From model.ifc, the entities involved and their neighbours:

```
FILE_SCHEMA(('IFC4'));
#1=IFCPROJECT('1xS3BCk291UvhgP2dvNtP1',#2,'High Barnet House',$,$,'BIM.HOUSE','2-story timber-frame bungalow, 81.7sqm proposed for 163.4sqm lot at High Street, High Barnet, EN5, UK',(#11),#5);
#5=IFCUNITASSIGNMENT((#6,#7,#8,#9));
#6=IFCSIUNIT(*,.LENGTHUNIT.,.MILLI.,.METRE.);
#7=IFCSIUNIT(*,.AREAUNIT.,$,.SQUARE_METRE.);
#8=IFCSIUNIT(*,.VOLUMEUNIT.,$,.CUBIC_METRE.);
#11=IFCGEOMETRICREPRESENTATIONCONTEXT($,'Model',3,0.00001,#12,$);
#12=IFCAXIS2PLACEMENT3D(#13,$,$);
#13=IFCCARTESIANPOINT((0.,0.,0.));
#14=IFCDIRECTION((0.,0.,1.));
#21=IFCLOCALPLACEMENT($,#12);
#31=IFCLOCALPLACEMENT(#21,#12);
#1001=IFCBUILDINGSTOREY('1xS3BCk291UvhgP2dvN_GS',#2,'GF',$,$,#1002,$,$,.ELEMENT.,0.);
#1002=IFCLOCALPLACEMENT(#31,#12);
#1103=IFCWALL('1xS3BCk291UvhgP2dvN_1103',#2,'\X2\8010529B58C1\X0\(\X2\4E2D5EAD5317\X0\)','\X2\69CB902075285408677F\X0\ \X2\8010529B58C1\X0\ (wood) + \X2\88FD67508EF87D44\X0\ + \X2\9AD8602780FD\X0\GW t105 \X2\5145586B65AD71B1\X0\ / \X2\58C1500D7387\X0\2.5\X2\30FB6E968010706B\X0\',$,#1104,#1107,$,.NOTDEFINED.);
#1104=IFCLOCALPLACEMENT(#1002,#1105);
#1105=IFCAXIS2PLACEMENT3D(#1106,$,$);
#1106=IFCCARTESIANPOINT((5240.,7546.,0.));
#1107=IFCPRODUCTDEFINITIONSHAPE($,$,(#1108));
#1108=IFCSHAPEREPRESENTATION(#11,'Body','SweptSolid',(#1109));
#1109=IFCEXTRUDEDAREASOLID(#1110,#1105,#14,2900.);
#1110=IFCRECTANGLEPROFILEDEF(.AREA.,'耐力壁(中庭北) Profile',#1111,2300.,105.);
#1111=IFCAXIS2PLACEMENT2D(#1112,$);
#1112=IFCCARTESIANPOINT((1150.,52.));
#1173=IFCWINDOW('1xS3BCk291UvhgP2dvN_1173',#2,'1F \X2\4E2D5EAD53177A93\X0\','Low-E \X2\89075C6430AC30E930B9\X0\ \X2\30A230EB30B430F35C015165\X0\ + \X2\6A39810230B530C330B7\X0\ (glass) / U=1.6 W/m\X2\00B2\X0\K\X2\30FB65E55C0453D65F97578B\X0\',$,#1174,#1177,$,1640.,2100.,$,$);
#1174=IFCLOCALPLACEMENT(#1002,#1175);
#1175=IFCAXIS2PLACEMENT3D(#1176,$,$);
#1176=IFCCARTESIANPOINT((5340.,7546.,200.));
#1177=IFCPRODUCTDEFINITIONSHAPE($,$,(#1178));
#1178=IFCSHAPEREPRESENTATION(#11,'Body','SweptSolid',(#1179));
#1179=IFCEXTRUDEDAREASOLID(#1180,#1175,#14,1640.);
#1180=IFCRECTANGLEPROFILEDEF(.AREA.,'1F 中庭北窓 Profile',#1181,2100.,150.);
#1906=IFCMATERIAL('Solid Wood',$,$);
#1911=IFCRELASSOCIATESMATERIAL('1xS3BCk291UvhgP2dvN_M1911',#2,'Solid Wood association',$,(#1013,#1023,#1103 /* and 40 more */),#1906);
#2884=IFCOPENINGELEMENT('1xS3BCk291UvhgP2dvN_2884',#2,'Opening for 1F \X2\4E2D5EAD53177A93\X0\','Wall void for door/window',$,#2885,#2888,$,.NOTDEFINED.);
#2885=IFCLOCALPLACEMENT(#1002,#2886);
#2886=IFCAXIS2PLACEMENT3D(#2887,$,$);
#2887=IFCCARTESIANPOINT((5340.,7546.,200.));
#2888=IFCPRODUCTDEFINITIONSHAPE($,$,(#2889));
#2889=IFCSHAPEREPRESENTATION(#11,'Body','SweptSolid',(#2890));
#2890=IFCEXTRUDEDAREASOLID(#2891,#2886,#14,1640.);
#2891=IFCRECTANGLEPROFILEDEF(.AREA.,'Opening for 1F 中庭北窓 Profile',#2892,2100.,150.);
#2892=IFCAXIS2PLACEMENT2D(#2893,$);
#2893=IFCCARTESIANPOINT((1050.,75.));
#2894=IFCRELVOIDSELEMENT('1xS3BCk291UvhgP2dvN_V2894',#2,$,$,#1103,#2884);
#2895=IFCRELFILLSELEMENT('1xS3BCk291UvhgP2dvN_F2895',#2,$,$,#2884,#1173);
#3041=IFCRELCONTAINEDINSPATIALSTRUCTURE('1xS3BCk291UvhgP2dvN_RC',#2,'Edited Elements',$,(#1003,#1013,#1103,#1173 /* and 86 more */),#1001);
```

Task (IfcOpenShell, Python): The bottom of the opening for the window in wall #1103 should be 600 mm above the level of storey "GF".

```python
import numpy as np
import ifcopenshell
import ifcopenshell.api.geometry
import ifcopenshell.geom
import ifcopenshell.util.element
import ifcopenshell.util.placement
import ifcopenshell.util.shape
import ifcopenshell.util.unit

model = ifcopenshell.open("model.ifc")
unit_scale = ifcopenshell.util.unit.calculate_unit_scale(model)

window = model.by_guid("1xS3BCk291UvhgP2dvN_1173")
opening = window.FillsVoids[0].RelatingOpeningElement
storey = ifcopenshell.util.element.get_container(window, ifc_class="IfcBuildingStorey")
level = ifcopenshell.util.placement.get_local_placement(storey.ObjectPlacement)[2, 3]

# The opening's origin need not be at the sill, so measure its lowest point.
shape = ifcopenshell.geom.create_shape(ifcopenshell.geom.settings(), opening)
bottom = ifcopenshell.util.shape.get_shape_bottom_elevation(shape, shape.geometry) / unit_scale
dz = level + 600.0 - bottom

shift = np.array([0.0, 0.0, dz])
# The window is not placed relative to its opening, so move both.
for product in (opening, window):
    matrix = ifcopenshell.util.placement.get_local_placement(product.ObjectPlacement)
    matrix[:3, 3] += shift
    ifcopenshell.api.geometry.edit_object_placement(model, product=product, matrix=matrix, is_si=False)

print(f"moved by {dz * unit_scale:+.3f} m")

model.write("model_edited.ifc")
```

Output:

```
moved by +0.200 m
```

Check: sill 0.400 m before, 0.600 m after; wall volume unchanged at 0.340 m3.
